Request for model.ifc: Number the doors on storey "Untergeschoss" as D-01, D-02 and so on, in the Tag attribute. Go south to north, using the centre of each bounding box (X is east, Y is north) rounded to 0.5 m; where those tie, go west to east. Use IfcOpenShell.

First a look at what the model holds.

```python
import ifcopenshell
import ifcopenshell.util.element
import ifcopenshell.util.placement

model = ifcopenshell.open("model.ifc")
print(model.schema)
storey = next(s for s in model.by_type("IfcBuildingStorey") if s.Name == "Untergeschoss")
doors = [e for e in ifcopenshell.util.element.get_decomposition(storey) if e.is_a("IfcDoor")]
for e in sorted(doors, key=lambda e: e.id()):
    origin = ifcopenshell.util.placement.get_local_placement(e.ObjectPlacement)[:3, 3]
    print(e.id(), e.Tag, e.Name, origin.round(2) + 0.0, sep=" | ")
```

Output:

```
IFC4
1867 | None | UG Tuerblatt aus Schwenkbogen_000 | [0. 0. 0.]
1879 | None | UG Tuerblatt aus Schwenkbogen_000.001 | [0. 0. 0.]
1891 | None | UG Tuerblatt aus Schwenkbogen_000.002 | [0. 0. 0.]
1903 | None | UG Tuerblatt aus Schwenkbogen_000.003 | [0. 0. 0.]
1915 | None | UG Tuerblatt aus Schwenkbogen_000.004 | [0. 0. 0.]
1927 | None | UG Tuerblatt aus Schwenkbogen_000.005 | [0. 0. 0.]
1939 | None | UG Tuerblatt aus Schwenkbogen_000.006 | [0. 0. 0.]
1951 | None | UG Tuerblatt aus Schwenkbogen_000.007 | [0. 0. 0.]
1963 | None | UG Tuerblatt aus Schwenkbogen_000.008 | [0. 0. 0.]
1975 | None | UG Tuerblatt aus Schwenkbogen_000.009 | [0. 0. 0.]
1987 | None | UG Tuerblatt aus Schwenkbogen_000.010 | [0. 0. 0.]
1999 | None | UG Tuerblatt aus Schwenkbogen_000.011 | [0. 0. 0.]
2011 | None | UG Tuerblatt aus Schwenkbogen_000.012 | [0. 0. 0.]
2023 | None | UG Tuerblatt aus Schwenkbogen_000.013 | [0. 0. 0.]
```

```python
import ifcopenshell
import ifcopenshell.geom
import ifcopenshell.util.element
import ifcopenshell.util.shape

model = ifcopenshell.open("model.ifc")
settings = ifcopenshell.geom.settings()
settings.set("use-world-coords", True)


def centre(element):
    shape = ifcopenshell.geom.create_shape(settings, element)
    return ifcopenshell.util.shape.get_bbox_centroid(shape.geometry)


storey = next(s for s in model.by_type("IfcBuildingStorey") if s.Name == "Untergeschoss")
doors = [e for e in ifcopenshell.util.element.get_decomposition(storey) if e.is_a("IfcDoor")]

# Insertion points can sit at a corner or the storey origin, so sort by the geometry (in metres).
centres = {e: centre(e) for e in doors}
doors.sort(key=lambda e: (round(centres[e][1] / 0.5), centres[e][0]))

for i, e in enumerate(doors, start=1):
    number = f"D-{i:02d}"
    e.Tag = number
    print(e.id(), number)

model.write("model_rev.ifc")
```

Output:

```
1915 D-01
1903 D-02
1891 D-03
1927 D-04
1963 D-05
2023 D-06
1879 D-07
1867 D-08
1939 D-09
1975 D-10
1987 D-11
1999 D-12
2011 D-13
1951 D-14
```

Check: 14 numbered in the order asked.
